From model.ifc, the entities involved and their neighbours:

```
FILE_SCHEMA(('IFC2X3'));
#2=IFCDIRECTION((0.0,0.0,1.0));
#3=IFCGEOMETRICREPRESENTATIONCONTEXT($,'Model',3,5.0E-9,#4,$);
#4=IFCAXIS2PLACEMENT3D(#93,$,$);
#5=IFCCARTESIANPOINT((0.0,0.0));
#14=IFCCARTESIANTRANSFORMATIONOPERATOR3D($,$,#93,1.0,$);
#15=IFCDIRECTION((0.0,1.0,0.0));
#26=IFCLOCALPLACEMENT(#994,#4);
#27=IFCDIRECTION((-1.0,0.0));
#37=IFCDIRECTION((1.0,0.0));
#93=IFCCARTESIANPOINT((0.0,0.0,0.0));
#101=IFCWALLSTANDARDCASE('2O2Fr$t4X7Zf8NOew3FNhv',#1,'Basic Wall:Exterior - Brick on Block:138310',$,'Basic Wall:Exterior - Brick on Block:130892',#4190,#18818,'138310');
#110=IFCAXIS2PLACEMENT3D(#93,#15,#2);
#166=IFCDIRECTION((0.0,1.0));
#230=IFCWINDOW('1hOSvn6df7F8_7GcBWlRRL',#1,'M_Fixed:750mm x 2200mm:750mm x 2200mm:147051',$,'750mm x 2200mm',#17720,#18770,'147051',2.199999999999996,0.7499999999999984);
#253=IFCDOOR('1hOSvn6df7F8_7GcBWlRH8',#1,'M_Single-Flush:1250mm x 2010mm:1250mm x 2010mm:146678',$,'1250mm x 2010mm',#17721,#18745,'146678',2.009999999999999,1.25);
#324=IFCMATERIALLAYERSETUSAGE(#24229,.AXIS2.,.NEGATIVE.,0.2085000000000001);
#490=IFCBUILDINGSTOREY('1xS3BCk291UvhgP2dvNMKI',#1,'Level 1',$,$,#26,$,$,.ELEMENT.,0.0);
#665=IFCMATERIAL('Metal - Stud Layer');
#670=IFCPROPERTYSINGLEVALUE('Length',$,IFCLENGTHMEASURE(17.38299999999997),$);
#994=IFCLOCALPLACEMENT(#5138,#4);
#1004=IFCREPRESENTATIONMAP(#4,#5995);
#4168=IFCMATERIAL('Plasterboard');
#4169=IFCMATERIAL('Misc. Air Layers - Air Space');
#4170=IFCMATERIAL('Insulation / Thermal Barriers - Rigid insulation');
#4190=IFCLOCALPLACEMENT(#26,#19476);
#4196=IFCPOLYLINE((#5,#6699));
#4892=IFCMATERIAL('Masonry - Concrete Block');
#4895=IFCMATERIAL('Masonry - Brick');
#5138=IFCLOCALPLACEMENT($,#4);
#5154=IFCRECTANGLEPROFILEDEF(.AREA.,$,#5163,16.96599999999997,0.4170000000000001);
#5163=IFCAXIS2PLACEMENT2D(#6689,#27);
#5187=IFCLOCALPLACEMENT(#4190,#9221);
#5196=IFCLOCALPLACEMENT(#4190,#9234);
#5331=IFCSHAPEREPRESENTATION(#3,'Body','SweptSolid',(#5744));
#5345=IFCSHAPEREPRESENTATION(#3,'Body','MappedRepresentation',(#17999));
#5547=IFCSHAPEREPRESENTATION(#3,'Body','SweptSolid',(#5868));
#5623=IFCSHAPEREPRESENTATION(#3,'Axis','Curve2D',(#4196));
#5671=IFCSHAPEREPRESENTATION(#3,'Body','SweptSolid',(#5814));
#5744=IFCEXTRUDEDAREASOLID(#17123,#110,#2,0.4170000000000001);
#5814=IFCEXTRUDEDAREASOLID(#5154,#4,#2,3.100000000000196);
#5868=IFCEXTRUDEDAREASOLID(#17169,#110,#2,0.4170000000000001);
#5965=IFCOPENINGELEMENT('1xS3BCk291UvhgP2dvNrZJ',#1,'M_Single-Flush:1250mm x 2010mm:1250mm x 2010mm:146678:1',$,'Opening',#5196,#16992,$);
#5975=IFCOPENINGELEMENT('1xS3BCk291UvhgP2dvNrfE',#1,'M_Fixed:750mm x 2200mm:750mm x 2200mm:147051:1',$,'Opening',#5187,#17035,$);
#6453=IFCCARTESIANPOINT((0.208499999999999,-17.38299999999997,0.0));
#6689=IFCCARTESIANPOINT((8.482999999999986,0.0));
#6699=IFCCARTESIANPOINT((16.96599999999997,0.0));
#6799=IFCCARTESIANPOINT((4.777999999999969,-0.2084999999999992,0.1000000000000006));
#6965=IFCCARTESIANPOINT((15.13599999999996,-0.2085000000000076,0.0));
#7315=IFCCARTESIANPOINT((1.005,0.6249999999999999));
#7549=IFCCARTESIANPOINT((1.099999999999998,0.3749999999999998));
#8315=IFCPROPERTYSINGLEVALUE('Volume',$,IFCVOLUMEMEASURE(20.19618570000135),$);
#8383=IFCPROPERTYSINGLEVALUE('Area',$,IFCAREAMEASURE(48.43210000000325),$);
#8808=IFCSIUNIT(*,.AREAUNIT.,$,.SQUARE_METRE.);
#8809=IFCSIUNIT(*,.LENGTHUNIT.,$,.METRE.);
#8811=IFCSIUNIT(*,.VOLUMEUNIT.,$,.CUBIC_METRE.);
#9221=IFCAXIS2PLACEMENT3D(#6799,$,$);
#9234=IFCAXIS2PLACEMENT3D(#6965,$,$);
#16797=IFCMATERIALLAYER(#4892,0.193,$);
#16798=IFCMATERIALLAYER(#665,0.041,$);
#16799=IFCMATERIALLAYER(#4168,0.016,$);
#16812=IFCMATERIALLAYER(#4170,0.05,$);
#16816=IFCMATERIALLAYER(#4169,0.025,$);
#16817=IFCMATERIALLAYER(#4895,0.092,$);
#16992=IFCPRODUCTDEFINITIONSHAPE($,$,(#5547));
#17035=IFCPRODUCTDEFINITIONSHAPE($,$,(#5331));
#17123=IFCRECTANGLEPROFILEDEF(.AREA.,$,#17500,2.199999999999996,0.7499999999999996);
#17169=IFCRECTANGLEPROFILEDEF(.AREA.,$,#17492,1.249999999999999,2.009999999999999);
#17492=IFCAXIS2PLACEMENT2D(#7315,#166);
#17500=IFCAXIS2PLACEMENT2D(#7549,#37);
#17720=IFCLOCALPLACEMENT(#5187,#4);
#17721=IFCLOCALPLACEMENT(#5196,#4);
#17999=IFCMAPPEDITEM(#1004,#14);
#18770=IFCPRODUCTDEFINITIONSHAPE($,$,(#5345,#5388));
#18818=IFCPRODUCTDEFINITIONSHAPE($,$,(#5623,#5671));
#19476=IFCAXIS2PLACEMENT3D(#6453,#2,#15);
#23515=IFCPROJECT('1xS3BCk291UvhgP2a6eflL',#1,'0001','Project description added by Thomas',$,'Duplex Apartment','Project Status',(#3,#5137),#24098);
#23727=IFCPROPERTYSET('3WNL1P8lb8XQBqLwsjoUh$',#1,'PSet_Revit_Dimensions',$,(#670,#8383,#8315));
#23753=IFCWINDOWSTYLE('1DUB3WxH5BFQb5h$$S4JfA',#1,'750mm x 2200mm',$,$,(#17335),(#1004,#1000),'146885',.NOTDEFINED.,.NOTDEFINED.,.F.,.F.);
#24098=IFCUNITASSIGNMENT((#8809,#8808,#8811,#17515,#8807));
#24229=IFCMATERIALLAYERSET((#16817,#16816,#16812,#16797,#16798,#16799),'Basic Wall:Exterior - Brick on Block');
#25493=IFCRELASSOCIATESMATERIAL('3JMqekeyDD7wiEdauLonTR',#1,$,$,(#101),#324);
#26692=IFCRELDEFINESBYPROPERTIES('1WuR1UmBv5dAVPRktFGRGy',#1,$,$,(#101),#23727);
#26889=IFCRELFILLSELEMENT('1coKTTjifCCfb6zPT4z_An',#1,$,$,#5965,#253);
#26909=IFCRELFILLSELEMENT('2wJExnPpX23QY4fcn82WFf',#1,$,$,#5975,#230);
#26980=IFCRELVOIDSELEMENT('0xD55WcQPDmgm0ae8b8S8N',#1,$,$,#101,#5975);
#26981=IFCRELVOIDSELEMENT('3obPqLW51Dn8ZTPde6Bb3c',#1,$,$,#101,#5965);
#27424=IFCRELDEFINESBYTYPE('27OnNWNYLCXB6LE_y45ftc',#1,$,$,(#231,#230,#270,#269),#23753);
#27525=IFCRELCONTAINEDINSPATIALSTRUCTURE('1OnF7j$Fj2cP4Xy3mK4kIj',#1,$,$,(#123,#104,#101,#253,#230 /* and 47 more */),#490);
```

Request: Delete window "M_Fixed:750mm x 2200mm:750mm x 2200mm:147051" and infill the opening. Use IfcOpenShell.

```python
import ifcopenshell
import ifcopenshell.api.feature
import ifcopenshell.api.pset
import ifcopenshell.api.root
import ifcopenshell.geom
import ifcopenshell.util.element
import ifcopenshell.util.shape
import ifcopenshell.util.unit

model = ifcopenshell.open("model.ifc")
area_scale = ifcopenshell.util.unit.calculate_unit_scale(model, "AREAUNIT")
volume_scale = ifcopenshell.util.unit.calculate_unit_scale(model, "VOLUMEUNIT")
settings = ifcopenshell.geom.settings()


def volume(element):
    """Net volume in cubic metres, openings subtracted."""
    shape = ifcopenshell.geom.create_shape(settings, element)
    return ifcopenshell.util.shape.get_volume(shape.geometry)


window = model.by_guid("1hOSvn6df7F8_7GcBWlRRL")
opening = window.FillsVoids[0].RelatingOpeningElement
wall = opening.VoidsElements[0].RelatingBuildingElement
before = volume(wall)

ifcopenshell.api.root.remove_product(model, product=window)
ifcopenshell.api.feature.remove_feature(model, feature=opening)

after = volume(wall)
thickness = 0.417  # wall thickness in metres

# Update the wall's stored quantities.
pset = model.by_id(ifcopenshell.util.element.get_pset(wall, "PSet_Revit_Dimensions", should_inherit=False)["id"])
ifcopenshell.api.pset.edit_pset(model, pset=pset, properties={
    "Area": model.create_entity("IfcAreaMeasure", after / thickness / area_scale),
    "Volume": model.create_entity("IfcVolumeMeasure", after / volume_scale),
})

print(f"wall volume {before:.3f} -> {after:.3f} m3")

model.write("model_v2.ifc")
```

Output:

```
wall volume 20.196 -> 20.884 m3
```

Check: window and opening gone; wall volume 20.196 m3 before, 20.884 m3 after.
